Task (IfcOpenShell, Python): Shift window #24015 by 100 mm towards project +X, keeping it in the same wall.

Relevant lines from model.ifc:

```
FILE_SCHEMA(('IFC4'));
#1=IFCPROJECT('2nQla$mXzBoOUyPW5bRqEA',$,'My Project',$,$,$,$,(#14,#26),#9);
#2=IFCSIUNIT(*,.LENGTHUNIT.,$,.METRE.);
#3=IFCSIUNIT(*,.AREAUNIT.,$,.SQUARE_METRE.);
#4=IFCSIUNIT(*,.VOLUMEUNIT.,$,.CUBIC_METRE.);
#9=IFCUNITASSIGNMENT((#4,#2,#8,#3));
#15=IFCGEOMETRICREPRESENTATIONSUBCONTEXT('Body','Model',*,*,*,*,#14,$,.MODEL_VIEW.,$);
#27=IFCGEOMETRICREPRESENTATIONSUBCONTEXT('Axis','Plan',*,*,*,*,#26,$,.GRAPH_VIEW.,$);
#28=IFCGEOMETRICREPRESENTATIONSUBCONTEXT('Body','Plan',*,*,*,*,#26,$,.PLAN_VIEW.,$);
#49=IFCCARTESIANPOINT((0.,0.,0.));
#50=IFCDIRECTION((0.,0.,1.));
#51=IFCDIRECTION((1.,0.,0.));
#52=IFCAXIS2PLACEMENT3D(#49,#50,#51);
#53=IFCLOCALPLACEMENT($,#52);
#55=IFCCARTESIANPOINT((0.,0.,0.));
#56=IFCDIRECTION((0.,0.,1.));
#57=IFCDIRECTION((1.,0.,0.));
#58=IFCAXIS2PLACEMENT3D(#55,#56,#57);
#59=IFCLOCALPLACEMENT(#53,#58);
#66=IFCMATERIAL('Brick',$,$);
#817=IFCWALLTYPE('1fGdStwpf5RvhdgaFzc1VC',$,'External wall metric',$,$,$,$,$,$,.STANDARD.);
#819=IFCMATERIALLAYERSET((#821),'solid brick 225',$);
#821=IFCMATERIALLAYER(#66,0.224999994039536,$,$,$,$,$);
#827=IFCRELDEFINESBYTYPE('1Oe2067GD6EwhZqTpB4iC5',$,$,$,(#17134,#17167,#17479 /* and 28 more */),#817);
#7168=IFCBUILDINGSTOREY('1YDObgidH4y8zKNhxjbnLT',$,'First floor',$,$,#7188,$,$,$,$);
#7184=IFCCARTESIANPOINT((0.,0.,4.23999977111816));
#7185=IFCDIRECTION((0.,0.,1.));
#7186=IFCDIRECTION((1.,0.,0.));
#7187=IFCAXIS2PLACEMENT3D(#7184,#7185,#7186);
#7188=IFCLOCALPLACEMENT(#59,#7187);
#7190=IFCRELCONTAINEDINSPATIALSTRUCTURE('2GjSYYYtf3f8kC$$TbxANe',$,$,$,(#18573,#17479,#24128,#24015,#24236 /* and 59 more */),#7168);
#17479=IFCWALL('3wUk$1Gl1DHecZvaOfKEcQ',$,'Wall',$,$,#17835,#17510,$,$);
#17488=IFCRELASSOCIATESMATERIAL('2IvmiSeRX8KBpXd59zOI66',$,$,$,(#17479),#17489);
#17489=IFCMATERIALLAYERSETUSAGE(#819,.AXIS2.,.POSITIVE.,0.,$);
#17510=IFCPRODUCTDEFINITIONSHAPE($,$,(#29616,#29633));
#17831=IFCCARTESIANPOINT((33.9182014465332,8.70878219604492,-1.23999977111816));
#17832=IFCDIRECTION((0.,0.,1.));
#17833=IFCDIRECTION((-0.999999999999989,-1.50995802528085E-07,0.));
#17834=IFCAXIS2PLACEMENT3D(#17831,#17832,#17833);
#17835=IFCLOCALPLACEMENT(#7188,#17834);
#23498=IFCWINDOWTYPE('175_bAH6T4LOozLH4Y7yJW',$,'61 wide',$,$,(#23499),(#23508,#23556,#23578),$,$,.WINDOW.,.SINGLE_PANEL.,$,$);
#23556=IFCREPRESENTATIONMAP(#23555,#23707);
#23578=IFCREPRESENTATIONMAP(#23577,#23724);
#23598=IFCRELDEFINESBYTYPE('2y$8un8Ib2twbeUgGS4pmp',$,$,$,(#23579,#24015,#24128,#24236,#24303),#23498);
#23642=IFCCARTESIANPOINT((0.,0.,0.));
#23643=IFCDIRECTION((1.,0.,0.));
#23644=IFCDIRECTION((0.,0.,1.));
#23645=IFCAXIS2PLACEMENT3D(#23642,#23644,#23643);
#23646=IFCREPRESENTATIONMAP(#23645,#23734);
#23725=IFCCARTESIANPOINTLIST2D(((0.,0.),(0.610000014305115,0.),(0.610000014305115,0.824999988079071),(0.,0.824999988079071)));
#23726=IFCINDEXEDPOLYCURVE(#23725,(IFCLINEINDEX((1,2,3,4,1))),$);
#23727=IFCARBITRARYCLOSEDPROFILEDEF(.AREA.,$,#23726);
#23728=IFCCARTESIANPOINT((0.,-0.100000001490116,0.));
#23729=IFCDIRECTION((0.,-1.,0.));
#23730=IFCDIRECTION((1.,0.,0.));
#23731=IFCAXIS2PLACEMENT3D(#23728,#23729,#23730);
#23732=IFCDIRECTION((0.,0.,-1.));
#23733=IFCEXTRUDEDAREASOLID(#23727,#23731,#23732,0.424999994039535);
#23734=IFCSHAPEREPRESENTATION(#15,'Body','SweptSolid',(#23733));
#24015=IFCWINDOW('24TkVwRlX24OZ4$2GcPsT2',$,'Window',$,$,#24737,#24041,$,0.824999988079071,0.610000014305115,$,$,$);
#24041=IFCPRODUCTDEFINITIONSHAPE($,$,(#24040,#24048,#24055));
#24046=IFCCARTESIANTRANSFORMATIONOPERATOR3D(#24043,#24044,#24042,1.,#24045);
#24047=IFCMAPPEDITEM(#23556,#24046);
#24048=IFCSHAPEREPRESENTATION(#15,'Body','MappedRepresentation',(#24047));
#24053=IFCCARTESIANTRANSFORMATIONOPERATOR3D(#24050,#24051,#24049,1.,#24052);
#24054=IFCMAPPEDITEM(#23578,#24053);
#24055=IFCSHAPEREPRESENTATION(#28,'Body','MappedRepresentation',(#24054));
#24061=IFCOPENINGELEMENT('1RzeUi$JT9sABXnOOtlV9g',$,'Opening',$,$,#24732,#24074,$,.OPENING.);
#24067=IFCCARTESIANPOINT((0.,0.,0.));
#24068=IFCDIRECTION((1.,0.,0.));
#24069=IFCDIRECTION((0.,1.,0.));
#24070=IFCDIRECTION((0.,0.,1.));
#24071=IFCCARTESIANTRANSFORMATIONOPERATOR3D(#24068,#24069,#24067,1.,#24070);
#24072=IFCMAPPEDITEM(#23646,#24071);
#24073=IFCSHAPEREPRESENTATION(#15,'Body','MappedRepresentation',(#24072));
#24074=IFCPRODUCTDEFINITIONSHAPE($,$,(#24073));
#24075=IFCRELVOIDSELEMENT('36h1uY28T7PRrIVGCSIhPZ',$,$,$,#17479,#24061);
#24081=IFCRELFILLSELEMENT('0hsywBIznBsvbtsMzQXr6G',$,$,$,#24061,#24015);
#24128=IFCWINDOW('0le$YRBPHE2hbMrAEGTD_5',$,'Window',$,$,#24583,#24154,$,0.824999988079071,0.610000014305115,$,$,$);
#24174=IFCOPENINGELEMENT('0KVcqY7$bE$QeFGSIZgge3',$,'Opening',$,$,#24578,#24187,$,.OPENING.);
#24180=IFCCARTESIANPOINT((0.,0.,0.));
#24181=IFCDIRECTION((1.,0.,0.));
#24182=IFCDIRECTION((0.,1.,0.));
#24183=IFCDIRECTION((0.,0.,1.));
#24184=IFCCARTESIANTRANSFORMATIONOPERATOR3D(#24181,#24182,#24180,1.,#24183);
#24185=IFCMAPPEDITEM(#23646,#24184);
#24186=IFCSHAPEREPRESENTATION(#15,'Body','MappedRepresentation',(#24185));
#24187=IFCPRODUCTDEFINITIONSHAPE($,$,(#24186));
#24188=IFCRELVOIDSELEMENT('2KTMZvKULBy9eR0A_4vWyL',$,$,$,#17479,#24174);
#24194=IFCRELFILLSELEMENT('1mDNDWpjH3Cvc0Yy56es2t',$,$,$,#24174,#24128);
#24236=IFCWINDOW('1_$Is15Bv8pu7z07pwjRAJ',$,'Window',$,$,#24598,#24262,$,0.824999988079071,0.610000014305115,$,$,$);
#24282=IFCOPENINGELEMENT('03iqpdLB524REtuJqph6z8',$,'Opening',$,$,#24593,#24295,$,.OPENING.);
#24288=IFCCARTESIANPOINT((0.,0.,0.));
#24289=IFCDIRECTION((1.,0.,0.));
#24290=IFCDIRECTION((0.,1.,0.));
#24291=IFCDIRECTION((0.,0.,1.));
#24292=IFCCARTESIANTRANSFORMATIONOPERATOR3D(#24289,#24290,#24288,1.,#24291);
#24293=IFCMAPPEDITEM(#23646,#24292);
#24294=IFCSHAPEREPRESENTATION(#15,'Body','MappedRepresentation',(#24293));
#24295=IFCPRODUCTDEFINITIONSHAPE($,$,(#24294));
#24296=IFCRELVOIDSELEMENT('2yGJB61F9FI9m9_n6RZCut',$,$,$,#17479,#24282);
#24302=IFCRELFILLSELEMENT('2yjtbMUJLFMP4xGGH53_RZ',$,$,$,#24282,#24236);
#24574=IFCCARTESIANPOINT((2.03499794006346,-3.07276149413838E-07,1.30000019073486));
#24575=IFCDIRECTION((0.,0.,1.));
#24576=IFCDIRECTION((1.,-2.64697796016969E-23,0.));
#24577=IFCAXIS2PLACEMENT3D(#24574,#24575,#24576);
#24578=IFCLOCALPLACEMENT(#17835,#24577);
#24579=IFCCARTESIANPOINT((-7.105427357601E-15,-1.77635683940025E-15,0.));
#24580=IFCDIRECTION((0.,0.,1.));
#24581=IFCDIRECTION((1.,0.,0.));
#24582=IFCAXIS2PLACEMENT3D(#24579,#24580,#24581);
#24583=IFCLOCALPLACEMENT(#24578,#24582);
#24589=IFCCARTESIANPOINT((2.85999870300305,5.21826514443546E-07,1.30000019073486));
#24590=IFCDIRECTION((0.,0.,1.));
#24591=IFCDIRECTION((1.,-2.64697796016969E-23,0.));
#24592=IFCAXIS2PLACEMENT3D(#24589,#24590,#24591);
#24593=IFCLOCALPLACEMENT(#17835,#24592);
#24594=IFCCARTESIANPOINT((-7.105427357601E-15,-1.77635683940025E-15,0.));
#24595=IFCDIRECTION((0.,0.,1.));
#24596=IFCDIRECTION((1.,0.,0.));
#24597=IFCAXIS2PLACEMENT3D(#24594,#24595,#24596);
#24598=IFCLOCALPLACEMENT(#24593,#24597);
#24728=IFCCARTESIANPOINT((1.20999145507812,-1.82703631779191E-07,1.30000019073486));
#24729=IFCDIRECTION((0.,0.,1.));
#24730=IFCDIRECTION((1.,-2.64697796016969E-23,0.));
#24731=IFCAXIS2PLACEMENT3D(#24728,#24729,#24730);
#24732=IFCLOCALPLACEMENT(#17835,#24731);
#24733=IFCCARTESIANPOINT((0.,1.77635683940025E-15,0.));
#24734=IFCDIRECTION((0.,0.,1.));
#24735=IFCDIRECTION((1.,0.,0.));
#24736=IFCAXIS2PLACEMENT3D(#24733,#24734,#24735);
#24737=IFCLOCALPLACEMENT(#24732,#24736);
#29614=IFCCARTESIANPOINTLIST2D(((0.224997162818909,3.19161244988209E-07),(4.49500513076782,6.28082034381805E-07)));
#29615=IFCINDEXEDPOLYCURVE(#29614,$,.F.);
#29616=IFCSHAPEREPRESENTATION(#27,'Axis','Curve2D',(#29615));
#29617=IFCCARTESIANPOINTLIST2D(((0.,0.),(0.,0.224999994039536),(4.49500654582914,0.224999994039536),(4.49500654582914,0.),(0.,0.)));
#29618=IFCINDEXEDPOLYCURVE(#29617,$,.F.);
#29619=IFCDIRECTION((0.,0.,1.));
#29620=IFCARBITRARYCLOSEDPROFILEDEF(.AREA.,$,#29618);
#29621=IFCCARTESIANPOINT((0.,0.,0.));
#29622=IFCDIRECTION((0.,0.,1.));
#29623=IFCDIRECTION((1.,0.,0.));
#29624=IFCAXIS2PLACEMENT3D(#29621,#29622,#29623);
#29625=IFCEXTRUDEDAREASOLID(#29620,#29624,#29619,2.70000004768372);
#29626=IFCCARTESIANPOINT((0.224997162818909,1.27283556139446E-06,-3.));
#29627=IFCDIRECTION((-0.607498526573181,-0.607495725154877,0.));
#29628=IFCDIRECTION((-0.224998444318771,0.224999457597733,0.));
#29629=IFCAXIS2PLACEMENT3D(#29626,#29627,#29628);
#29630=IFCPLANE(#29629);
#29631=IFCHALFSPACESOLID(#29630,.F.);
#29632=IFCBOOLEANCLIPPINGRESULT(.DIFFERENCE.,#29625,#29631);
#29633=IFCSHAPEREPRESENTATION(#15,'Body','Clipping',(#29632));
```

```python
import ifcopenshell
import ifcopenshell.api.geometry
import ifcopenshell.util.placement

model = ifcopenshell.open("model.ifc")

window = model.by_id(24015)
opening = window.FillsVoids[0].RelatingOpeningElement
wall = opening.VoidsElements[0].RelatingBuildingElement

wall_matrix = ifcopenshell.util.placement.get_local_placement(wall.ObjectPlacement)
shift = wall_matrix[:3, 0] * -0.1
before = ifcopenshell.util.placement.get_local_placement(window.ObjectPlacement)[:3, 3].copy()

# The window is placed relative to its opening, so it follows when the opening moves.
matrix = ifcopenshell.util.placement.get_local_placement(opening.ObjectPlacement)
matrix[:3, 3] += shift
ifcopenshell.api.geometry.edit_object_placement(
    model, product=opening, matrix=matrix, is_si=False, should_transform_children=True
)

after = ifcopenshell.util.placement.get_local_placement(window.ObjectPlacement)[:3, 3]
print("window moved by", (after - before).round(3) + 0.0)

model.write("model_updated.ifc")
```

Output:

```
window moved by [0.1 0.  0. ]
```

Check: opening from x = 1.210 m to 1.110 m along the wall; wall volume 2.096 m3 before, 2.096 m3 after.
